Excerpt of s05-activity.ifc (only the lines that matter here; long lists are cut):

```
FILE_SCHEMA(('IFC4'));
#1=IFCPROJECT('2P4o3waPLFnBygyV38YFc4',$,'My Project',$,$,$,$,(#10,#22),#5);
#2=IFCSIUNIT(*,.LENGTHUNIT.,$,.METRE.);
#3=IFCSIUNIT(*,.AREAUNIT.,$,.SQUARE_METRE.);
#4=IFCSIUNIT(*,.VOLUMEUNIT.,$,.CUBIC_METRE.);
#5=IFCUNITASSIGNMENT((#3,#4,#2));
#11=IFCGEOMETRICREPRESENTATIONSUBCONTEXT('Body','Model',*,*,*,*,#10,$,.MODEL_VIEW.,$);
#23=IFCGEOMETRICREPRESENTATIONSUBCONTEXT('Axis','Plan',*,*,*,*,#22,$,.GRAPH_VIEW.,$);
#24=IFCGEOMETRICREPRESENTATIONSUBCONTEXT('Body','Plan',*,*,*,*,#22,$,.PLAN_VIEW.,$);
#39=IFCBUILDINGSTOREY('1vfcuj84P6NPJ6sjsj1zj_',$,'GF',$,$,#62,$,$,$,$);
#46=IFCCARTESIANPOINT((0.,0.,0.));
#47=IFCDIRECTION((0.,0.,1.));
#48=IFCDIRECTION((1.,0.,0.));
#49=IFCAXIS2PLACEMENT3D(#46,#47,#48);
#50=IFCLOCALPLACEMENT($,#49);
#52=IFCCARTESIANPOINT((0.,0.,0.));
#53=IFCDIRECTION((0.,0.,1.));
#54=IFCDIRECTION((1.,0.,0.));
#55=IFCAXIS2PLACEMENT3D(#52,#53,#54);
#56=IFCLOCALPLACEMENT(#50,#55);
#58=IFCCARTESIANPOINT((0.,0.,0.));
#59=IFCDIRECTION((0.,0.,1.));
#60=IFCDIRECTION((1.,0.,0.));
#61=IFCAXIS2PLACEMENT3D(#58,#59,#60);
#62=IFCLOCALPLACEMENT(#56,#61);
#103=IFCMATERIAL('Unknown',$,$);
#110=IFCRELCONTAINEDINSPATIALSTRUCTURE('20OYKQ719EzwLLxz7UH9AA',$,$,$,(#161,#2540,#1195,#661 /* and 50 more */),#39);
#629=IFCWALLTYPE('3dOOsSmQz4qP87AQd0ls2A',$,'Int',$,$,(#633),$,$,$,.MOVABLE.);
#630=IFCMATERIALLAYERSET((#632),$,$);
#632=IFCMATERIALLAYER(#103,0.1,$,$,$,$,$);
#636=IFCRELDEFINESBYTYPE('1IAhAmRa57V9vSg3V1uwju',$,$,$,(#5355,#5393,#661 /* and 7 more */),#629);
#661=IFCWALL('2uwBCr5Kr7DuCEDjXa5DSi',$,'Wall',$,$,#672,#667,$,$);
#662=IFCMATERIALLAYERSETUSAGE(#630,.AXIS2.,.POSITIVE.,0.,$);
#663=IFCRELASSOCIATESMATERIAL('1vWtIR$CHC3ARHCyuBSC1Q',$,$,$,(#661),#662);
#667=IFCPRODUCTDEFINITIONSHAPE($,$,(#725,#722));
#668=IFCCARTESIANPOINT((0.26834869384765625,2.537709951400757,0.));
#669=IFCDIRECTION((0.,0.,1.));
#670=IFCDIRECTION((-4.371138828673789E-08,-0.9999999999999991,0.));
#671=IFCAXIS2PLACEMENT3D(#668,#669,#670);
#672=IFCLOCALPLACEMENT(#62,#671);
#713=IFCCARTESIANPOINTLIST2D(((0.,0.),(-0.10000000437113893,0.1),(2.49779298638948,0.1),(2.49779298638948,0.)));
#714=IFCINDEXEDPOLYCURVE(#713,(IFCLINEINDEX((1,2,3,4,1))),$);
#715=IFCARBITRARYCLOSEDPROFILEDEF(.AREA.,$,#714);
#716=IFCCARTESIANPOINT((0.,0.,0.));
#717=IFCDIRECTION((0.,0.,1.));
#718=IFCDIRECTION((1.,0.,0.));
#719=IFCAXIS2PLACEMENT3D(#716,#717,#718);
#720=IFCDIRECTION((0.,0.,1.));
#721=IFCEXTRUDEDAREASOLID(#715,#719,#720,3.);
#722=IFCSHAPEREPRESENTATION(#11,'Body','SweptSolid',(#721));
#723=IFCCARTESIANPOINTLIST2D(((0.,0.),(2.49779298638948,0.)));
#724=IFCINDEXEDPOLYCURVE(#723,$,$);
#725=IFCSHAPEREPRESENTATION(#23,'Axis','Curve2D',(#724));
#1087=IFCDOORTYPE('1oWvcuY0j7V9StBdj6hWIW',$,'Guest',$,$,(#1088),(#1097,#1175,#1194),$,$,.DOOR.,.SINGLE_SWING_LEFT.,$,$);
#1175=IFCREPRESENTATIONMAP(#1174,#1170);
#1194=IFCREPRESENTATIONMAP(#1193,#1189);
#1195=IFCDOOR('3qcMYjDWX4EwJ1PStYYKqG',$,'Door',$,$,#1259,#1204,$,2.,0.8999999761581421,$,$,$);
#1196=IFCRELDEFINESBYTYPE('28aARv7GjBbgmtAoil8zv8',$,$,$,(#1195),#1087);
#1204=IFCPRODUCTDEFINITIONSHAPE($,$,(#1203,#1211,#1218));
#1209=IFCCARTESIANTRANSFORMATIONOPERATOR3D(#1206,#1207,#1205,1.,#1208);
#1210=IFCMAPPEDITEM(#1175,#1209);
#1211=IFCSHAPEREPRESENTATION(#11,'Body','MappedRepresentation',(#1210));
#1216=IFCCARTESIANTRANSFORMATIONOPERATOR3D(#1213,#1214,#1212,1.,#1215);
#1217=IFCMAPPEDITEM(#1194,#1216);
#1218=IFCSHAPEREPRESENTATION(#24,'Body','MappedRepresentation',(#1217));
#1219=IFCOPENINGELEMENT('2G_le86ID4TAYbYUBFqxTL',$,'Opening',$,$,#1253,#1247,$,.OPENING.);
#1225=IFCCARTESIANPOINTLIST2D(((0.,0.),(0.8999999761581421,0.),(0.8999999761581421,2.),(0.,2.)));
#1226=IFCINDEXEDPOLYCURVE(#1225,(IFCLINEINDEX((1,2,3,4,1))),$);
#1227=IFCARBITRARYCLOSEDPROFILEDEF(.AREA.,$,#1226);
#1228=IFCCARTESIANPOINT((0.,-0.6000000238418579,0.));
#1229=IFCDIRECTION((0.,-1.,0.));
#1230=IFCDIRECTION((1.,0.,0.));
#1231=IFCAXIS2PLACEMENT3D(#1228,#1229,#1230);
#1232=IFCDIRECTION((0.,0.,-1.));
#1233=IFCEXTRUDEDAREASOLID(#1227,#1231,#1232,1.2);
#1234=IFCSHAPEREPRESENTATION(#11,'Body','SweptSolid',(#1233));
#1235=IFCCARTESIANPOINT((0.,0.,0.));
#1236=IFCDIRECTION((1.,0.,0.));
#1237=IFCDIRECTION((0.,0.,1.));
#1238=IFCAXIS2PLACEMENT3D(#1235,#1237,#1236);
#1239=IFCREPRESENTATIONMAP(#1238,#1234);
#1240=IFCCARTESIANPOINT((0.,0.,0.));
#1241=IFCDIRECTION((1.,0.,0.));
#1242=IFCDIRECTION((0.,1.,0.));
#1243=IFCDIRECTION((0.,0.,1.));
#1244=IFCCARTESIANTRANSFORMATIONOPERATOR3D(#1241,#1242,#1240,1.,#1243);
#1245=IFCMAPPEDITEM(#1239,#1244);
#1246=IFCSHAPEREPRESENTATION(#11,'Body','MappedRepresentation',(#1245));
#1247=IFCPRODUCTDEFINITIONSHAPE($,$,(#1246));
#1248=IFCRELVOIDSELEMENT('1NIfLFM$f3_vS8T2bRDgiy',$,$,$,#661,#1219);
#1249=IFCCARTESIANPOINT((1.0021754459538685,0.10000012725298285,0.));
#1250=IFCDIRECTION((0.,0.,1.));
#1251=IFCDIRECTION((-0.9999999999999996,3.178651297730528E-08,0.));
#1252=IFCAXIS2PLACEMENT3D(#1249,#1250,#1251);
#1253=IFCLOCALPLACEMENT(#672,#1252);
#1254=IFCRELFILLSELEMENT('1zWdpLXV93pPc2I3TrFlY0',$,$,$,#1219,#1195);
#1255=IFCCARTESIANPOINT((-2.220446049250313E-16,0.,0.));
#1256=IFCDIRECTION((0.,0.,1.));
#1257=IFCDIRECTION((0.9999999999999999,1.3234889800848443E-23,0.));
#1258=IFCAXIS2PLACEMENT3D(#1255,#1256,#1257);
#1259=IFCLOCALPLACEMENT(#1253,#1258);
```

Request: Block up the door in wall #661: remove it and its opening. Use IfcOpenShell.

```python
import ifcopenshell
import ifcopenshell.api.feature
import ifcopenshell.api.root
import ifcopenshell.geom
import ifcopenshell.util.shape

model = ifcopenshell.open("s05-activity.ifc")
settings = ifcopenshell.geom.settings()


def volume(element):
    """Net volume in cubic metres, openings subtracted."""
    shape = ifcopenshell.geom.create_shape(settings, element)
    return ifcopenshell.util.shape.get_volume(shape.geometry)


door = model.by_guid("3qcMYjDWX4EwJ1PStYYKqG")
opening = door.FillsVoids[0].RelatingOpeningElement
wall = opening.VoidsElements[0].RelatingBuildingElement
before = volume(wall)

ifcopenshell.api.root.remove_product(model, product=door)
ifcopenshell.api.feature.remove_feature(model, feature=opening)

after = volume(wall)

print(f"wall volume {before:.3f} -> {after:.3f} m3")

model.write("s05-activity_v2.ifc")
```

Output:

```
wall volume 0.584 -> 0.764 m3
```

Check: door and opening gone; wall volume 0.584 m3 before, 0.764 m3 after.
